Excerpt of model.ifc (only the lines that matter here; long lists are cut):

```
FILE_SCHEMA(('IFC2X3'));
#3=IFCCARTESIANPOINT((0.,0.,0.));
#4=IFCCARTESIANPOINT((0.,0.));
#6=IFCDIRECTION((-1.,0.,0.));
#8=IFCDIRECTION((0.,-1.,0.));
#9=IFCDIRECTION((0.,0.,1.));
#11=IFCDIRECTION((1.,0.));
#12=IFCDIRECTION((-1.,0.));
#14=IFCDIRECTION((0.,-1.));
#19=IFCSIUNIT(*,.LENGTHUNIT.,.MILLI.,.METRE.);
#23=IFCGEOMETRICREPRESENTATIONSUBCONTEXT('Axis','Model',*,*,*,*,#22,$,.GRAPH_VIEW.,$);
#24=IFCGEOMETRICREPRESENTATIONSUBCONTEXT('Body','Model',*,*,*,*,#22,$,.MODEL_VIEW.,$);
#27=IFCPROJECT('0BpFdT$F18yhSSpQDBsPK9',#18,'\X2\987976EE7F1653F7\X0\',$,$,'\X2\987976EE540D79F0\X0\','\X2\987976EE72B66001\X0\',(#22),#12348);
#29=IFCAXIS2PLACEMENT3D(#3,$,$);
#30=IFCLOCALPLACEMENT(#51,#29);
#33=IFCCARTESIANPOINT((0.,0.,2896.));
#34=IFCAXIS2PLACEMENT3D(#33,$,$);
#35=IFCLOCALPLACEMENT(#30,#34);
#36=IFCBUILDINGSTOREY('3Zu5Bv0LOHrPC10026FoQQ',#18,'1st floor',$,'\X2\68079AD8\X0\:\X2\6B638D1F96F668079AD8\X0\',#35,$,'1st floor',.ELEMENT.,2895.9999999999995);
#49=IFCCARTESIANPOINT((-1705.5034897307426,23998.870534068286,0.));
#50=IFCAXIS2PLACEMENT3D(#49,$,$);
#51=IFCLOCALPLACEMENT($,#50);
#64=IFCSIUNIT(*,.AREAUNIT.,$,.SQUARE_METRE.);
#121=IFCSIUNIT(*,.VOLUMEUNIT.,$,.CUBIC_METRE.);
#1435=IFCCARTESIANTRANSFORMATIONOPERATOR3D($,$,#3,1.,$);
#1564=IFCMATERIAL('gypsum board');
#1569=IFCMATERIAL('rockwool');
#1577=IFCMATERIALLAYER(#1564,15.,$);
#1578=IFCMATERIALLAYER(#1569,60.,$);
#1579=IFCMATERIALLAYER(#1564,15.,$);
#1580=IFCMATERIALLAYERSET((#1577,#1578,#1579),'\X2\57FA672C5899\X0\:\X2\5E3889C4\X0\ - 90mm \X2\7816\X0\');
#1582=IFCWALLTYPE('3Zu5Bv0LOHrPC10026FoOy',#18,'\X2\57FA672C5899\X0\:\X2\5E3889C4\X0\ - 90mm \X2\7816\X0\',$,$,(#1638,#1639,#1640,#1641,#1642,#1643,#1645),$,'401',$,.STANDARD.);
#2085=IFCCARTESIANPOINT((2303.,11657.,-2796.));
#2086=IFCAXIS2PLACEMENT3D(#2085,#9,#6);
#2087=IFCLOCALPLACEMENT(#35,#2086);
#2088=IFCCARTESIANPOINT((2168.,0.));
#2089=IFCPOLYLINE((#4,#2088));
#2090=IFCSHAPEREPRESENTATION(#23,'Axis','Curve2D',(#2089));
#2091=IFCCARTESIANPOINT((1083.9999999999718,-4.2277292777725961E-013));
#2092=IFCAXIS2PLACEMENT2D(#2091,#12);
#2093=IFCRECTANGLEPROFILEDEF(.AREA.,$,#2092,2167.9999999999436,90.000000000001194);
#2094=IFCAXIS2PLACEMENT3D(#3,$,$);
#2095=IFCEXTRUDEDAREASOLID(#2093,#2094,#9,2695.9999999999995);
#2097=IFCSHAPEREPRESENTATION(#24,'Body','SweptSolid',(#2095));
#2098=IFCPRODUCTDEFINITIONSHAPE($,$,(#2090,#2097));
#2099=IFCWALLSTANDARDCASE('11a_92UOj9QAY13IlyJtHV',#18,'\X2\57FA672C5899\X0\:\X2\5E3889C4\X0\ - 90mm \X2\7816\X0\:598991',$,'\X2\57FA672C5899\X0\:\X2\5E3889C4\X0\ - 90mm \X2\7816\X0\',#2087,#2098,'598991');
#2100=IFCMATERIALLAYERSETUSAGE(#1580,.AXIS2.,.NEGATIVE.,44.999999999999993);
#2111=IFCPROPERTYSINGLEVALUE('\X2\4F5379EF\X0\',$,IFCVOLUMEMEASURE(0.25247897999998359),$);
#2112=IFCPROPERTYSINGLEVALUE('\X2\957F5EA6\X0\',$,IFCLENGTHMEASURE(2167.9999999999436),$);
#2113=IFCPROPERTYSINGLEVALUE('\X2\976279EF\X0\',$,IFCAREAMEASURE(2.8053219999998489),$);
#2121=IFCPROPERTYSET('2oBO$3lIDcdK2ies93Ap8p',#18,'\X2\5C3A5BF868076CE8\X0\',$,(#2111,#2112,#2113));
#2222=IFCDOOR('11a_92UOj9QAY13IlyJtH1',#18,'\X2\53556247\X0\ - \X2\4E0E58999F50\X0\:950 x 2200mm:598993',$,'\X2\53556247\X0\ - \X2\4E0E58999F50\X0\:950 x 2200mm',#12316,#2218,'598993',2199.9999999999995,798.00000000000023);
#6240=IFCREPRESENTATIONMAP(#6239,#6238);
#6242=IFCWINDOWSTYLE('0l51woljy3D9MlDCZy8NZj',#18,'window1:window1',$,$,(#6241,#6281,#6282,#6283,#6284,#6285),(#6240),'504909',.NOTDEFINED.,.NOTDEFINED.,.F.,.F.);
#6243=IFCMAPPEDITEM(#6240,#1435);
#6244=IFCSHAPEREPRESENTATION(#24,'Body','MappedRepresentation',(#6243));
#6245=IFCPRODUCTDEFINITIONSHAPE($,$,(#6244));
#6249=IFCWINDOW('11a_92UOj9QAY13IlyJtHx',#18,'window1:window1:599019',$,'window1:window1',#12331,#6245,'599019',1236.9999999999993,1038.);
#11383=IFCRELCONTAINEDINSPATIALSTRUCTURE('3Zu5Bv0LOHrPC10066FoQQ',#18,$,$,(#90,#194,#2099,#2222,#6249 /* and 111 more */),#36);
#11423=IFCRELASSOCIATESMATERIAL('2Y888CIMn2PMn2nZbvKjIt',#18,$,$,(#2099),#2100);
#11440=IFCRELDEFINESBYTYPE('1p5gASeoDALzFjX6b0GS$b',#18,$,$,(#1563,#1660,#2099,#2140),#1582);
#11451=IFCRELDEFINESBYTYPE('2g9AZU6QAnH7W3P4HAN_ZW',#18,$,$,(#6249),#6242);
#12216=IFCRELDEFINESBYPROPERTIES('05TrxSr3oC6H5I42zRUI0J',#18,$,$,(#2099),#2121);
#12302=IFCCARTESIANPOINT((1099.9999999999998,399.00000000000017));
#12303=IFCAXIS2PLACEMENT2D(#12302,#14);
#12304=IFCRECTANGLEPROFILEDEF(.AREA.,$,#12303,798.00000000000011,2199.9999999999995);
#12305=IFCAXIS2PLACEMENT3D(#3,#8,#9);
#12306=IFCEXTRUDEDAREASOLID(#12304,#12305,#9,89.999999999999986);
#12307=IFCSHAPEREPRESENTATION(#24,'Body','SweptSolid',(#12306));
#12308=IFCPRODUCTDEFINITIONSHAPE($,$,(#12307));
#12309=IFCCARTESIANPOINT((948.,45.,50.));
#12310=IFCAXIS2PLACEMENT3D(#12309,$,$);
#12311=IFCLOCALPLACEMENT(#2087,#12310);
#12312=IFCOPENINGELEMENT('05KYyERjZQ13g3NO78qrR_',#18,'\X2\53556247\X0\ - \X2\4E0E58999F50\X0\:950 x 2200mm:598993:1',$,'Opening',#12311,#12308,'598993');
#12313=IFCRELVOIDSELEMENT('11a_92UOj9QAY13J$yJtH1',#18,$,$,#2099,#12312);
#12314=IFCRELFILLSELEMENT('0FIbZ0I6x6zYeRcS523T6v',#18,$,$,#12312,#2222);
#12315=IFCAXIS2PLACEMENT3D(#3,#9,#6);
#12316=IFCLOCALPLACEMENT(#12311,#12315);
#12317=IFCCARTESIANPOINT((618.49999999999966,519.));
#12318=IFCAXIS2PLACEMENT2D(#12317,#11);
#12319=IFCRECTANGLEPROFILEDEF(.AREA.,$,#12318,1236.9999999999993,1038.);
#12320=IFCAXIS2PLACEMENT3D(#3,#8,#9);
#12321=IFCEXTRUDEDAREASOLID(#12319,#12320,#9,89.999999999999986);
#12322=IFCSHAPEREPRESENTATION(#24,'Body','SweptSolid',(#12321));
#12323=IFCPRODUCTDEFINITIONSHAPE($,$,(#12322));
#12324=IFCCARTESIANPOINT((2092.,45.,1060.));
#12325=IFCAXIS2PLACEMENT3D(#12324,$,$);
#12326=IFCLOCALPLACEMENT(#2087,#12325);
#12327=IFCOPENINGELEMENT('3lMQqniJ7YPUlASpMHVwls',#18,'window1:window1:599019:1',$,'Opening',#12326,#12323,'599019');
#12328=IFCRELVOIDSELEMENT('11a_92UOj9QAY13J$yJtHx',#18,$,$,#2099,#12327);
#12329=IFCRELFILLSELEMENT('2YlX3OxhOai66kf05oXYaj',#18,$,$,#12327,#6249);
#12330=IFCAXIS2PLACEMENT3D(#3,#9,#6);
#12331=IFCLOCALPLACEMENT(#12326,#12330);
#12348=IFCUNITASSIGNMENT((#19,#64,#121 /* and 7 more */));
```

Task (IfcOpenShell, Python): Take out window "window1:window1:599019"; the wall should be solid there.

```python
import ifcopenshell
import ifcopenshell.api.feature
import ifcopenshell.api.pset
import ifcopenshell.api.root
import ifcopenshell.geom
import ifcopenshell.util.element
import ifcopenshell.util.shape
import ifcopenshell.util.unit

model = ifcopenshell.open("model.ifc")
area_scale = ifcopenshell.util.unit.calculate_unit_scale(model, "AREAUNIT")
volume_scale = ifcopenshell.util.unit.calculate_unit_scale(model, "VOLUMEUNIT")
settings = ifcopenshell.geom.settings()


def volume(element):
    """Net volume in cubic metres, openings subtracted."""
    shape = ifcopenshell.geom.create_shape(settings, element)
    return ifcopenshell.util.shape.get_volume(shape.geometry)


window = model.by_guid("11a_92UOj9QAY13IlyJtHx")
opening = window.FillsVoids[0].RelatingOpeningElement
wall = opening.VoidsElements[0].RelatingBuildingElement
before = volume(wall)

ifcopenshell.api.root.remove_product(model, product=window)
ifcopenshell.api.feature.remove_feature(model, feature=opening)

after = volume(wall)
thickness = 0.09  # wall thickness in metres

# Update the wall's stored quantities.
pset = model.by_id(ifcopenshell.util.element.get_pset(wall, "尺寸标注", should_inherit=False)["id"])
ifcopenshell.api.pset.edit_pset(model, pset=pset, properties={
    "体积": model.create_entity("IfcVolumeMeasure", after / volume_scale),
    "面积": model.create_entity("IfcAreaMeasure", after / thickness / area_scale),
})

print(f"wall volume {before:.3f} -> {after:.3f} m3")

model.write("model-out.ifc")
```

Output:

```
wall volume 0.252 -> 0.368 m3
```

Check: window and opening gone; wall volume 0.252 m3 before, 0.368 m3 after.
